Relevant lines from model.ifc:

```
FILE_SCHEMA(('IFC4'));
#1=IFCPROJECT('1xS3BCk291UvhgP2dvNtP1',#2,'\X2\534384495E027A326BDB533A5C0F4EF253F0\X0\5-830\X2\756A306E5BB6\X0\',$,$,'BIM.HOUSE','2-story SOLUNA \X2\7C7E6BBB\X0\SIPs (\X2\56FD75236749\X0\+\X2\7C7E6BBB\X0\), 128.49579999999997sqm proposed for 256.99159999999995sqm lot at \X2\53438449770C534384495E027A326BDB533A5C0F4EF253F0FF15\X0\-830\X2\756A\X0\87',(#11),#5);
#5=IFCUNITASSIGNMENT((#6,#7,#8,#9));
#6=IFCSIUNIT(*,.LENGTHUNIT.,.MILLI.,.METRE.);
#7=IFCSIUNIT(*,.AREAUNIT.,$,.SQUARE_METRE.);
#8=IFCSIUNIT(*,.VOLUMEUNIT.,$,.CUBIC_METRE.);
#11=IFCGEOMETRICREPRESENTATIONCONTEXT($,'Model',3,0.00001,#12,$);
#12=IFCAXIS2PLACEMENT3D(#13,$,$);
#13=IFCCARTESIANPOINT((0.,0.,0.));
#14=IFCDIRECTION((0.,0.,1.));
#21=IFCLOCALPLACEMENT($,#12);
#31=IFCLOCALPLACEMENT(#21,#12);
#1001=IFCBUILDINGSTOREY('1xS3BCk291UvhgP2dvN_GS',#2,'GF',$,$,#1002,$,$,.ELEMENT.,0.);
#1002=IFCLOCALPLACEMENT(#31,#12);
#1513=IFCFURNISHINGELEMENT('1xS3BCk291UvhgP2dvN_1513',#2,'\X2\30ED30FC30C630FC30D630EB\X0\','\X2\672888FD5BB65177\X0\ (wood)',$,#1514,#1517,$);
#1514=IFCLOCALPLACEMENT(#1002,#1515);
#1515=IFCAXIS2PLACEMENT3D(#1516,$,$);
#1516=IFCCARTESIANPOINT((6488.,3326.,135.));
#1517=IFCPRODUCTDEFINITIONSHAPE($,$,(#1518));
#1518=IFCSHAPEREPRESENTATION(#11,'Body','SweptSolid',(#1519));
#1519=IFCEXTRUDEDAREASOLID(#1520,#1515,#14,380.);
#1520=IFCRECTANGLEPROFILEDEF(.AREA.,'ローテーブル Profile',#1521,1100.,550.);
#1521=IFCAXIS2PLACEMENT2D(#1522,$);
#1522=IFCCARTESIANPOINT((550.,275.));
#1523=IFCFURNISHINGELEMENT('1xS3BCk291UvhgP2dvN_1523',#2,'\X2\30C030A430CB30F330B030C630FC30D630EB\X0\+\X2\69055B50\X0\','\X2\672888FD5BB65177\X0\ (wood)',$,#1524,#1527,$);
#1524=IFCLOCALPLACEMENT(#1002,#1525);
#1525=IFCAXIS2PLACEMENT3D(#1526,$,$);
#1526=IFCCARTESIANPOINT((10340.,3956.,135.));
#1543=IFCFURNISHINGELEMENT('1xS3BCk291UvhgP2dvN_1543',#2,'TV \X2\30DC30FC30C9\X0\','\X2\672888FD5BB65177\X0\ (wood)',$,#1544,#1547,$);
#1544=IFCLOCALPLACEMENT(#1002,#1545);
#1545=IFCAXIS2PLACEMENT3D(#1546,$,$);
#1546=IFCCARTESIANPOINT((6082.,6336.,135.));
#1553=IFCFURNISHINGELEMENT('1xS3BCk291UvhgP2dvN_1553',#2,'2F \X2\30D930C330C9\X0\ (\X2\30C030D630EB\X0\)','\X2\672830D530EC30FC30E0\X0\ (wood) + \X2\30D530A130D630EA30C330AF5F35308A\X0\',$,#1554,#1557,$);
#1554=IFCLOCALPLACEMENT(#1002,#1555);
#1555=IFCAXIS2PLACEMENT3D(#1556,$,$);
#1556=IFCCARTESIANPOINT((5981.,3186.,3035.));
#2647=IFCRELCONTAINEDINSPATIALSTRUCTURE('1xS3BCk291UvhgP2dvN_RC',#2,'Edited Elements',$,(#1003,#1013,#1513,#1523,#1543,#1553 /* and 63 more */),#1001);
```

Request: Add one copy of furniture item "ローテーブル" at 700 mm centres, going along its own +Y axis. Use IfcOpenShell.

```python
import ifcopenshell
import ifcopenshell.api.geometry
import ifcopenshell.api.root
import ifcopenshell.util.element
import ifcopenshell.util.placement

model = ifcopenshell.open("model.ifc")


def reuse_history(source, copy):
    """copy_class also copies each property set's owner history, people and application; keep the originals."""
    for rel in copy.IsDefinedBy:
        if rel.is_a("IfcRelDefinesByProperties") and (history := rel.RelatingPropertyDefinition.OwnerHistory):
            rel.RelatingPropertyDefinition.OwnerHistory = source.OwnerHistory
            ifcopenshell.util.element.remove_deep2(model, history)


source = model.by_guid("1xS3BCk291UvhgP2dvN_1513")
base = ifcopenshell.util.placement.get_local_placement(source.ObjectPlacement)
step = base[:3, 1] * 700.0

for i in range(1, 2):
    copy = ifcopenshell.api.root.copy_class(model, product=source)
    copy.Representation = ifcopenshell.util.element.copy_deep(
        model, source.Representation, exclude=["IfcGeometricRepresentationContext", "IfcRepresentationMap"]
    )
    reuse_history(source, copy)
    matrix = base.copy()
    matrix[:3, 3] += i * step
    print("added at", matrix[:3, 3].round(3) + 0.0)
    ifcopenshell.api.geometry.edit_object_placement(model, product=copy, matrix=matrix, is_si=False)

model.write("model_rev.ifc")
```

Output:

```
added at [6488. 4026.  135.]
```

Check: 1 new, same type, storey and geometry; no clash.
